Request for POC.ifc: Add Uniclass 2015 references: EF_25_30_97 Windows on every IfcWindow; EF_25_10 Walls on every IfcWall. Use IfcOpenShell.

First a look at what the model holds.

```python
import ifcopenshell

model = ifcopenshell.open("POC.ifc")
print(model.schema)
print("classifications:", [c.Name for c in model.by_type("IfcClassification")])
for ifc_class in ("IfcDoor", "IfcRoof", "IfcStair", "IfcWall", "IfcWindow"):
    print(ifc_class, len(model.by_type(ifc_class)))
```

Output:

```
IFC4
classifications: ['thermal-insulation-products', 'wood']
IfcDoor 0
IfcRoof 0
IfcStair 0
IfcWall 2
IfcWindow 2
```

```python
import ifcopenshell
import ifcopenshell.api.classification

model = ifcopenshell.open("POC.ifc")

system = ifcopenshell.api.classification.add_classification(model, classification="Uniclass 2015")

codes = {
    "IfcWindow": ("EF_25_30_97", "Windows"),
    "IfcWall": ("EF_25_10", "Walls"),
}
for ifc_class, (code, name) in codes.items():
    products = model.by_type(ifc_class)
    ifcopenshell.api.classification.add_reference(
        model, products=products, classification=system, identification=code, name=name
    )
    print(code, len(products))

model.write("POC_rev.ifc")
```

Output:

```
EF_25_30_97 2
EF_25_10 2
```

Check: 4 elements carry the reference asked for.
